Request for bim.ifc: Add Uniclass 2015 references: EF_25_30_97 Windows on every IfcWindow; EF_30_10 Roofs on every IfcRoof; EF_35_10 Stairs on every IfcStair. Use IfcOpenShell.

First a look at what the model holds.

```python
import ifcopenshell

model = ifcopenshell.open("bim.ifc")
print(model.schema)
print("classifications:", [c.Name for c in model.by_type("IfcClassification")])
for ifc_class in ("IfcDoor", "IfcRoof", "IfcStair", "IfcWall", "IfcWindow"):
    print(ifc_class, len(model.by_type(ifc_class)))
```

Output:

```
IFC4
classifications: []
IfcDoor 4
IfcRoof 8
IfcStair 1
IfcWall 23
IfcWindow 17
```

```python
import ifcopenshell
import ifcopenshell.api.classification

model = ifcopenshell.open("bim.ifc")

system = ifcopenshell.api.classification.add_classification(model, classification="Uniclass 2015")

codes = {
    "IfcWindow": ("EF_25_30_97", "Windows"),
    "IfcRoof": ("EF_30_10", "Roofs"),
    "IfcStair": ("EF_35_10", "Stairs"),
}
for ifc_class, (code, name) in codes.items():
    products = model.by_type(ifc_class)
    ifcopenshell.api.classification.add_reference(
        model, products=products, classification=system, identification=code, name=name
    )
    print(code, len(products))

model.write("bim_updated.ifc")
```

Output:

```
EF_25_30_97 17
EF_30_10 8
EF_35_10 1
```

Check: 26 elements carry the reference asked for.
